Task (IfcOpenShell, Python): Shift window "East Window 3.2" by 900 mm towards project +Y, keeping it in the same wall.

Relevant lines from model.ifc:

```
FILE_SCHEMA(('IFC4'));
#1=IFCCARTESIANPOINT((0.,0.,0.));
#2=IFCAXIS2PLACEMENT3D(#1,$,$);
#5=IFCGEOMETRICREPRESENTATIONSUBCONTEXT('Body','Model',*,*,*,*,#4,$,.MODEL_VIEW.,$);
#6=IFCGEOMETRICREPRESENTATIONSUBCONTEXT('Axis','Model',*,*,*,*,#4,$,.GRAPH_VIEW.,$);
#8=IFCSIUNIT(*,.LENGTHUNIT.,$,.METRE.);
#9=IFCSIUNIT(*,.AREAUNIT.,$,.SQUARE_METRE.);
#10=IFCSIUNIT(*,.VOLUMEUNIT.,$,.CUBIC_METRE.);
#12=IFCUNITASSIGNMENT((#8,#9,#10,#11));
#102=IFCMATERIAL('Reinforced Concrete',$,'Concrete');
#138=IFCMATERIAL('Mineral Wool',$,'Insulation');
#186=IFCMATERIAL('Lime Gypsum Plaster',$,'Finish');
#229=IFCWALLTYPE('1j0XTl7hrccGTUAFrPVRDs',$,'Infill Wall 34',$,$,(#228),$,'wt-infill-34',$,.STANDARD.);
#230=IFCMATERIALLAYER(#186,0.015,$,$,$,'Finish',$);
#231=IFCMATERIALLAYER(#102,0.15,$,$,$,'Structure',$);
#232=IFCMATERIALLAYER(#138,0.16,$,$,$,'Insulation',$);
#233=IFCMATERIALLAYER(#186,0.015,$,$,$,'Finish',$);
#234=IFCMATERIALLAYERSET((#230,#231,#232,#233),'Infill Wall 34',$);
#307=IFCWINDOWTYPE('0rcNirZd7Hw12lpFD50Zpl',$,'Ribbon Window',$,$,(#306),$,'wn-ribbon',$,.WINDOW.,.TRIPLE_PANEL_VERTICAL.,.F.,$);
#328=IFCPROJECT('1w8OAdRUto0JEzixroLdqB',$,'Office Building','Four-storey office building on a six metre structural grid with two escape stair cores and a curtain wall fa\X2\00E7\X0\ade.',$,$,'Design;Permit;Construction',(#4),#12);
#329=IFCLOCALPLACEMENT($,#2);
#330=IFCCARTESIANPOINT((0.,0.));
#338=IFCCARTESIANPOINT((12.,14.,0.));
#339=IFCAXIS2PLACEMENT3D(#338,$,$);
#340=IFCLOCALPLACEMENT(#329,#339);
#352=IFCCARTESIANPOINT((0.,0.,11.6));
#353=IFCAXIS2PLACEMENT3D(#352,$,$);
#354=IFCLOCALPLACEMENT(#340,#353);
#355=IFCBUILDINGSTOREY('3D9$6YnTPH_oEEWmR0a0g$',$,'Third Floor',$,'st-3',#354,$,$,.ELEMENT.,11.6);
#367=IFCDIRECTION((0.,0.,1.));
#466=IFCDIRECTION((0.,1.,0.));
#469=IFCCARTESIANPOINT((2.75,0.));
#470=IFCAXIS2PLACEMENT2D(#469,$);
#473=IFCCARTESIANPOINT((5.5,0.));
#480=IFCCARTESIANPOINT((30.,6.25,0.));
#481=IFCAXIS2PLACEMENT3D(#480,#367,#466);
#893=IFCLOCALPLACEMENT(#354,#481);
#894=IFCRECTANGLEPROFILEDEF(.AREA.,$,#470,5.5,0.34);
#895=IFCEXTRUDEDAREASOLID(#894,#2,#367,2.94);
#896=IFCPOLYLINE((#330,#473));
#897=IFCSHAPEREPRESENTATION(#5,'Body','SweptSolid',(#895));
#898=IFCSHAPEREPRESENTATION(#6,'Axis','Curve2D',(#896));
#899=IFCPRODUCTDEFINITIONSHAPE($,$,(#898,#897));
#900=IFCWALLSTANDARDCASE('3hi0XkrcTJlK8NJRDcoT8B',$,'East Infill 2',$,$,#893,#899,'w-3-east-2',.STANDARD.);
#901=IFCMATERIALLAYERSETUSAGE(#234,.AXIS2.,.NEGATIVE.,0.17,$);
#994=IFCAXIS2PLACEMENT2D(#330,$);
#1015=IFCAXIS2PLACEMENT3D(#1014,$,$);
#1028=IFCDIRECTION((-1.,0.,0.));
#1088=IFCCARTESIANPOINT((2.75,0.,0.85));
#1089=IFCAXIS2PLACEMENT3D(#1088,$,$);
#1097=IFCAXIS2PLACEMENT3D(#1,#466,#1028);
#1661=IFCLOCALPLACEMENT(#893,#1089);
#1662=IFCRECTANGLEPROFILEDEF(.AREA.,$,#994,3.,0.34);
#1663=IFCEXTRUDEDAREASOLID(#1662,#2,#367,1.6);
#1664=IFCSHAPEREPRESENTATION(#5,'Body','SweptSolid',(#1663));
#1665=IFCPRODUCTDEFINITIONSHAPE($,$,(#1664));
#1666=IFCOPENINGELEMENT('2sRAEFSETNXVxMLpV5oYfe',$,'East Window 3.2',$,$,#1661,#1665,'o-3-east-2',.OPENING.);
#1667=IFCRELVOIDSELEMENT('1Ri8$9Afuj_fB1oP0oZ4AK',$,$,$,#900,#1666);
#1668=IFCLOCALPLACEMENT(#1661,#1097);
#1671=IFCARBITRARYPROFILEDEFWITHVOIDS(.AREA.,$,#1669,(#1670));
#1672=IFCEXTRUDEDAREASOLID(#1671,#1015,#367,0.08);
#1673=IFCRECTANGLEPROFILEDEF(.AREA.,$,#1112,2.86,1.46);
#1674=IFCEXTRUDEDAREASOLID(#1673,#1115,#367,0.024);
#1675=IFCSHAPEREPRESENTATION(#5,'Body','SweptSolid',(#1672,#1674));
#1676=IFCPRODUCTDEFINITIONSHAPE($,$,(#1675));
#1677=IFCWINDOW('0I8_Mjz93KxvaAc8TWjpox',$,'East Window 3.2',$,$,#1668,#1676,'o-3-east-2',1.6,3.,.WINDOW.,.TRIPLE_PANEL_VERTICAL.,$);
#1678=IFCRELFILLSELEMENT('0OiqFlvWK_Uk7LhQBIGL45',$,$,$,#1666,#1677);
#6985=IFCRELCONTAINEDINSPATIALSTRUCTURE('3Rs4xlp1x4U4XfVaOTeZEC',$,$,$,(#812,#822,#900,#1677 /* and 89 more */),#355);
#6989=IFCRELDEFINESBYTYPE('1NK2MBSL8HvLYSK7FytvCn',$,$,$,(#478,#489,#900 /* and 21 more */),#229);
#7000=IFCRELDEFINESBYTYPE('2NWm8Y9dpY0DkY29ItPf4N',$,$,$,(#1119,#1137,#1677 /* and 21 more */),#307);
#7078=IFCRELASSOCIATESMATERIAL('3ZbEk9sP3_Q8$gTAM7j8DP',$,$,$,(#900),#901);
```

```python
import ifcopenshell
import ifcopenshell.api.geometry
import ifcopenshell.util.placement

model = ifcopenshell.open("model.ifc")

window = model.by_id(1677)
opening = window.FillsVoids[0].RelatingOpeningElement
wall = opening.VoidsElements[0].RelatingBuildingElement

wall_matrix = ifcopenshell.util.placement.get_local_placement(wall.ObjectPlacement)
shift = wall_matrix[:3, 0] * 0.9
before = ifcopenshell.util.placement.get_local_placement(window.ObjectPlacement)[:3, 3].copy()

# The window is placed relative to its opening, so it follows when the opening moves.
matrix = ifcopenshell.util.placement.get_local_placement(opening.ObjectPlacement)
matrix[:3, 3] += shift
ifcopenshell.api.geometry.edit_object_placement(
    model, product=opening, matrix=matrix, is_si=False, should_transform_children=True
)

after = ifcopenshell.util.placement.get_local_placement(window.ObjectPlacement)[:3, 3]
print("window moved by", (after - before).round(3) + 0.0)

model.write("model_rev.ifc")
```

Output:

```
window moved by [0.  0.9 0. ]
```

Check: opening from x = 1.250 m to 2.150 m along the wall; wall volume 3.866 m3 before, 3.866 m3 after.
